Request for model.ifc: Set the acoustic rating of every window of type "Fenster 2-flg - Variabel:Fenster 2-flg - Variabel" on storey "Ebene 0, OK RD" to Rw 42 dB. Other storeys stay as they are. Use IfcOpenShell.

First a look at what the model holds.

```python
import ifcopenshell
import ifcopenshell.util.element

model = ifcopenshell.open("model.ifc")
print(model.schema)
storey = next(s for s in model.by_type("IfcBuildingStorey") if s.Name == "Ebene 0, OK RD")
windows = [e for e in ifcopenshell.util.element.get_decomposition(storey) if e.is_a("IfcWindow")]
seen = {}
for e in windows:
    element_type = ifcopenshell.util.element.get_type(e)
    key = (element_type.Name if element_type != e and element_type else None, ifcopenshell.util.element.get_pset(e, "Pset_WindowCommon", "AcousticRating"))
    seen[key] = seen.get(key, 0) + 1
for (name, value), count in sorted(seen.items(), key=str):
    print(count, "x", name, "|", value)
```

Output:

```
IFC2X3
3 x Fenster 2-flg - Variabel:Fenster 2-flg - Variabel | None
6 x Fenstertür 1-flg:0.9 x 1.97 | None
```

```python
import ifcopenshell
import ifcopenshell.api.pset
import ifcopenshell.util.element

model = ifcopenshell.open("model.ifc")

storey = next(s for s in model.by_type("IfcBuildingStorey") if s.Name == "Ebene 0, OK RD")
windows = [e for e in ifcopenshell.util.element.get_decomposition(storey) if e.is_a("IfcWindow")]

count = 0
for e in windows:
    element_type = ifcopenshell.util.element.get_type(e)
    if element_type in (None, e) or element_type.Name != "Fenster 2-flg - Variabel:Fenster 2-flg - Variabel":
        continue
    # add_pset returns the element's existing set when there is one.
    pset = ifcopenshell.api.pset.add_pset(model, product=e, name="Pset_WindowCommon")
    ifcopenshell.api.pset.edit_pset(model, pset=pset, properties={"AcousticRating": "Rw 42 dB"})
    count += 1

print(count, "windows updated")

model.write("model-out.ifc")
```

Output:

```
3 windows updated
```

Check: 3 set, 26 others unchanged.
